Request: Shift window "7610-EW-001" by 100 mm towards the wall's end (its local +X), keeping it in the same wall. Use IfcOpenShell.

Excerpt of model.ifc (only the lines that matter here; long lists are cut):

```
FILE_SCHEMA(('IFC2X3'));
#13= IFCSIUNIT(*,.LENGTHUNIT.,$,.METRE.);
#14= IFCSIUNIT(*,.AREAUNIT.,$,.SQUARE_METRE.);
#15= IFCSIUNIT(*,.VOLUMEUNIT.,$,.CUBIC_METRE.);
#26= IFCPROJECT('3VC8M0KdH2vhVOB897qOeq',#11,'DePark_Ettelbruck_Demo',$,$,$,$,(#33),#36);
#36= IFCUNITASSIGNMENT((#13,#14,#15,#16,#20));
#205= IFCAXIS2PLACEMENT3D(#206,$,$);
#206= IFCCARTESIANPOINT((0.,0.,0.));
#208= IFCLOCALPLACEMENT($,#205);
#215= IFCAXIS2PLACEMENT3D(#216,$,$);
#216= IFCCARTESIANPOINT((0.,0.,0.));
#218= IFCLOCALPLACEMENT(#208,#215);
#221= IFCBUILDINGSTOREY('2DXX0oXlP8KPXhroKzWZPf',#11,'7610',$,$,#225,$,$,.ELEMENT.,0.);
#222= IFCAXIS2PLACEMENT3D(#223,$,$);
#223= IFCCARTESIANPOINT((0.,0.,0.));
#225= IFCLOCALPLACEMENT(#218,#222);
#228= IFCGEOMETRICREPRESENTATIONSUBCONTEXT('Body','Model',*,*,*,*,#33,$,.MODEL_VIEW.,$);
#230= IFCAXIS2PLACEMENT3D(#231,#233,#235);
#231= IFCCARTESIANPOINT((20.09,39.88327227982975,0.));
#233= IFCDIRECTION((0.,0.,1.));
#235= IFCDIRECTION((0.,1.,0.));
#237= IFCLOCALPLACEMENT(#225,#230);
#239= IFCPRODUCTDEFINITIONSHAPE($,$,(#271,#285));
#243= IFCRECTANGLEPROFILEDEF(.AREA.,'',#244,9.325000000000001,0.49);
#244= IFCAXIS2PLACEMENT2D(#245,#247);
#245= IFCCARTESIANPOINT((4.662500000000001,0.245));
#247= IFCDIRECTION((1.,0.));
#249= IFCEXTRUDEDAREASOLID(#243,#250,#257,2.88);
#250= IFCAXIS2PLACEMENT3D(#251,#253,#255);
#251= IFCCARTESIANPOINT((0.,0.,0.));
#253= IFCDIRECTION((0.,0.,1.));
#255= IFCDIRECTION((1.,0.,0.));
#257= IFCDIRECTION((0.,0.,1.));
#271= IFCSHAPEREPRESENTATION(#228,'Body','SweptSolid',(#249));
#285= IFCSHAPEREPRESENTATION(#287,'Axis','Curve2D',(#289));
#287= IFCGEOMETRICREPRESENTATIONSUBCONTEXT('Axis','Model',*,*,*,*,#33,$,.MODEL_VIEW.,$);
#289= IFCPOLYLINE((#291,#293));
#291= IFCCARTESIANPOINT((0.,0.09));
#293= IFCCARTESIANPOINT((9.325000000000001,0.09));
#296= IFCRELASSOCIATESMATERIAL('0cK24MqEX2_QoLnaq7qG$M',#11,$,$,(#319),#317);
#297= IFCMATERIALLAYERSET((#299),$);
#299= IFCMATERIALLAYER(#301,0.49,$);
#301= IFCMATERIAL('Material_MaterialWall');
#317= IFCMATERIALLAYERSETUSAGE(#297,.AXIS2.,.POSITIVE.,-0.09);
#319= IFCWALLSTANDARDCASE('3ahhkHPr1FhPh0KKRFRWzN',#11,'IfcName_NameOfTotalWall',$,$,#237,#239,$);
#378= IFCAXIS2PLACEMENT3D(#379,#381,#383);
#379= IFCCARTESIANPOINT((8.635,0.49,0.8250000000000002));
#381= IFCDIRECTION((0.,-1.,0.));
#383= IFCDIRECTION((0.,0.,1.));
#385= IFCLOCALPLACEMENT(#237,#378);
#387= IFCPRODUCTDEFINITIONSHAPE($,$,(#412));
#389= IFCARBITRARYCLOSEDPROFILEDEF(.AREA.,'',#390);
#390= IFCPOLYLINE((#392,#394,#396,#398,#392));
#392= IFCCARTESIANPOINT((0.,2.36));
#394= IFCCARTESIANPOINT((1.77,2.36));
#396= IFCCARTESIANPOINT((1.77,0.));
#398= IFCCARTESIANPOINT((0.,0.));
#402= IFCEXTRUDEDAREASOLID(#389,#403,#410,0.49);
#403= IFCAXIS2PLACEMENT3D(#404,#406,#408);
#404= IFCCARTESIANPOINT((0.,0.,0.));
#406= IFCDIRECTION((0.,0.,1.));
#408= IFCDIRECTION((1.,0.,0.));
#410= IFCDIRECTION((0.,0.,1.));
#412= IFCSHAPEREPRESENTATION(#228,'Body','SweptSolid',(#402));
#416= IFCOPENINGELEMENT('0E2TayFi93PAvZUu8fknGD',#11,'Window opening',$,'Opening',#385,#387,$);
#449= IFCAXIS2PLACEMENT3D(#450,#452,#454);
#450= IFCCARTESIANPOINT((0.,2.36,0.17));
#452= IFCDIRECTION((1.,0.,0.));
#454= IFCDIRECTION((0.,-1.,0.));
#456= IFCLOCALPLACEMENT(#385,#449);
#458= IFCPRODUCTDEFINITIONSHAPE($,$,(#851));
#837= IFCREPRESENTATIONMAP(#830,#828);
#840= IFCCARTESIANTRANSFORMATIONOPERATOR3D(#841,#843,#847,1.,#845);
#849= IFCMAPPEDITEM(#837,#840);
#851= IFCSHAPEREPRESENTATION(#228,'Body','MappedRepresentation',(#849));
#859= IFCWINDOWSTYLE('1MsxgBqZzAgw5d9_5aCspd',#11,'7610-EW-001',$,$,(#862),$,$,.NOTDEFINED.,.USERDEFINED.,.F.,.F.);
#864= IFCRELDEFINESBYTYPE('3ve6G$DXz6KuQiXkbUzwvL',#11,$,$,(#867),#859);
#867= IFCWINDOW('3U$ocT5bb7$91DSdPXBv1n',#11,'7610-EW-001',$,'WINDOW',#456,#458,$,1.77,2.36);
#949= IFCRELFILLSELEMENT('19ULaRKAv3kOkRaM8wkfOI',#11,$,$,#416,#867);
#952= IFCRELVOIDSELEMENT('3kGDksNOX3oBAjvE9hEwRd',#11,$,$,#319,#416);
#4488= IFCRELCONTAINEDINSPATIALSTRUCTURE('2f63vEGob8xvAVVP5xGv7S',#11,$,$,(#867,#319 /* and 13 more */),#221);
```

```python
import ifcopenshell
import ifcopenshell.api.geometry
import ifcopenshell.util.placement

model = ifcopenshell.open("model.ifc")

window = model.by_guid("3U$ocT5bb7$91DSdPXBv1n")
opening = window.FillsVoids[0].RelatingOpeningElement
wall = opening.VoidsElements[0].RelatingBuildingElement

wall_matrix = ifcopenshell.util.placement.get_local_placement(wall.ObjectPlacement)
shift = wall_matrix[:3, 0] * 0.1
before = ifcopenshell.util.placement.get_local_placement(window.ObjectPlacement)[:3, 3].copy()

# The window is placed relative to its opening, so it follows when the opening moves.
matrix = ifcopenshell.util.placement.get_local_placement(opening.ObjectPlacement)
matrix[:3, 3] += shift
ifcopenshell.api.geometry.edit_object_placement(
    model, product=opening, matrix=matrix, is_si=False, should_transform_children=True
)

after = ifcopenshell.util.placement.get_local_placement(window.ObjectPlacement)[:3, 3]
print("window moved by", (after - before).round(3) + 0.0)

model.write("model_v2.ifc")
```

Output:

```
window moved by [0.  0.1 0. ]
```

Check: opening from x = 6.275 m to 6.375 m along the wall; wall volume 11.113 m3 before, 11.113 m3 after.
